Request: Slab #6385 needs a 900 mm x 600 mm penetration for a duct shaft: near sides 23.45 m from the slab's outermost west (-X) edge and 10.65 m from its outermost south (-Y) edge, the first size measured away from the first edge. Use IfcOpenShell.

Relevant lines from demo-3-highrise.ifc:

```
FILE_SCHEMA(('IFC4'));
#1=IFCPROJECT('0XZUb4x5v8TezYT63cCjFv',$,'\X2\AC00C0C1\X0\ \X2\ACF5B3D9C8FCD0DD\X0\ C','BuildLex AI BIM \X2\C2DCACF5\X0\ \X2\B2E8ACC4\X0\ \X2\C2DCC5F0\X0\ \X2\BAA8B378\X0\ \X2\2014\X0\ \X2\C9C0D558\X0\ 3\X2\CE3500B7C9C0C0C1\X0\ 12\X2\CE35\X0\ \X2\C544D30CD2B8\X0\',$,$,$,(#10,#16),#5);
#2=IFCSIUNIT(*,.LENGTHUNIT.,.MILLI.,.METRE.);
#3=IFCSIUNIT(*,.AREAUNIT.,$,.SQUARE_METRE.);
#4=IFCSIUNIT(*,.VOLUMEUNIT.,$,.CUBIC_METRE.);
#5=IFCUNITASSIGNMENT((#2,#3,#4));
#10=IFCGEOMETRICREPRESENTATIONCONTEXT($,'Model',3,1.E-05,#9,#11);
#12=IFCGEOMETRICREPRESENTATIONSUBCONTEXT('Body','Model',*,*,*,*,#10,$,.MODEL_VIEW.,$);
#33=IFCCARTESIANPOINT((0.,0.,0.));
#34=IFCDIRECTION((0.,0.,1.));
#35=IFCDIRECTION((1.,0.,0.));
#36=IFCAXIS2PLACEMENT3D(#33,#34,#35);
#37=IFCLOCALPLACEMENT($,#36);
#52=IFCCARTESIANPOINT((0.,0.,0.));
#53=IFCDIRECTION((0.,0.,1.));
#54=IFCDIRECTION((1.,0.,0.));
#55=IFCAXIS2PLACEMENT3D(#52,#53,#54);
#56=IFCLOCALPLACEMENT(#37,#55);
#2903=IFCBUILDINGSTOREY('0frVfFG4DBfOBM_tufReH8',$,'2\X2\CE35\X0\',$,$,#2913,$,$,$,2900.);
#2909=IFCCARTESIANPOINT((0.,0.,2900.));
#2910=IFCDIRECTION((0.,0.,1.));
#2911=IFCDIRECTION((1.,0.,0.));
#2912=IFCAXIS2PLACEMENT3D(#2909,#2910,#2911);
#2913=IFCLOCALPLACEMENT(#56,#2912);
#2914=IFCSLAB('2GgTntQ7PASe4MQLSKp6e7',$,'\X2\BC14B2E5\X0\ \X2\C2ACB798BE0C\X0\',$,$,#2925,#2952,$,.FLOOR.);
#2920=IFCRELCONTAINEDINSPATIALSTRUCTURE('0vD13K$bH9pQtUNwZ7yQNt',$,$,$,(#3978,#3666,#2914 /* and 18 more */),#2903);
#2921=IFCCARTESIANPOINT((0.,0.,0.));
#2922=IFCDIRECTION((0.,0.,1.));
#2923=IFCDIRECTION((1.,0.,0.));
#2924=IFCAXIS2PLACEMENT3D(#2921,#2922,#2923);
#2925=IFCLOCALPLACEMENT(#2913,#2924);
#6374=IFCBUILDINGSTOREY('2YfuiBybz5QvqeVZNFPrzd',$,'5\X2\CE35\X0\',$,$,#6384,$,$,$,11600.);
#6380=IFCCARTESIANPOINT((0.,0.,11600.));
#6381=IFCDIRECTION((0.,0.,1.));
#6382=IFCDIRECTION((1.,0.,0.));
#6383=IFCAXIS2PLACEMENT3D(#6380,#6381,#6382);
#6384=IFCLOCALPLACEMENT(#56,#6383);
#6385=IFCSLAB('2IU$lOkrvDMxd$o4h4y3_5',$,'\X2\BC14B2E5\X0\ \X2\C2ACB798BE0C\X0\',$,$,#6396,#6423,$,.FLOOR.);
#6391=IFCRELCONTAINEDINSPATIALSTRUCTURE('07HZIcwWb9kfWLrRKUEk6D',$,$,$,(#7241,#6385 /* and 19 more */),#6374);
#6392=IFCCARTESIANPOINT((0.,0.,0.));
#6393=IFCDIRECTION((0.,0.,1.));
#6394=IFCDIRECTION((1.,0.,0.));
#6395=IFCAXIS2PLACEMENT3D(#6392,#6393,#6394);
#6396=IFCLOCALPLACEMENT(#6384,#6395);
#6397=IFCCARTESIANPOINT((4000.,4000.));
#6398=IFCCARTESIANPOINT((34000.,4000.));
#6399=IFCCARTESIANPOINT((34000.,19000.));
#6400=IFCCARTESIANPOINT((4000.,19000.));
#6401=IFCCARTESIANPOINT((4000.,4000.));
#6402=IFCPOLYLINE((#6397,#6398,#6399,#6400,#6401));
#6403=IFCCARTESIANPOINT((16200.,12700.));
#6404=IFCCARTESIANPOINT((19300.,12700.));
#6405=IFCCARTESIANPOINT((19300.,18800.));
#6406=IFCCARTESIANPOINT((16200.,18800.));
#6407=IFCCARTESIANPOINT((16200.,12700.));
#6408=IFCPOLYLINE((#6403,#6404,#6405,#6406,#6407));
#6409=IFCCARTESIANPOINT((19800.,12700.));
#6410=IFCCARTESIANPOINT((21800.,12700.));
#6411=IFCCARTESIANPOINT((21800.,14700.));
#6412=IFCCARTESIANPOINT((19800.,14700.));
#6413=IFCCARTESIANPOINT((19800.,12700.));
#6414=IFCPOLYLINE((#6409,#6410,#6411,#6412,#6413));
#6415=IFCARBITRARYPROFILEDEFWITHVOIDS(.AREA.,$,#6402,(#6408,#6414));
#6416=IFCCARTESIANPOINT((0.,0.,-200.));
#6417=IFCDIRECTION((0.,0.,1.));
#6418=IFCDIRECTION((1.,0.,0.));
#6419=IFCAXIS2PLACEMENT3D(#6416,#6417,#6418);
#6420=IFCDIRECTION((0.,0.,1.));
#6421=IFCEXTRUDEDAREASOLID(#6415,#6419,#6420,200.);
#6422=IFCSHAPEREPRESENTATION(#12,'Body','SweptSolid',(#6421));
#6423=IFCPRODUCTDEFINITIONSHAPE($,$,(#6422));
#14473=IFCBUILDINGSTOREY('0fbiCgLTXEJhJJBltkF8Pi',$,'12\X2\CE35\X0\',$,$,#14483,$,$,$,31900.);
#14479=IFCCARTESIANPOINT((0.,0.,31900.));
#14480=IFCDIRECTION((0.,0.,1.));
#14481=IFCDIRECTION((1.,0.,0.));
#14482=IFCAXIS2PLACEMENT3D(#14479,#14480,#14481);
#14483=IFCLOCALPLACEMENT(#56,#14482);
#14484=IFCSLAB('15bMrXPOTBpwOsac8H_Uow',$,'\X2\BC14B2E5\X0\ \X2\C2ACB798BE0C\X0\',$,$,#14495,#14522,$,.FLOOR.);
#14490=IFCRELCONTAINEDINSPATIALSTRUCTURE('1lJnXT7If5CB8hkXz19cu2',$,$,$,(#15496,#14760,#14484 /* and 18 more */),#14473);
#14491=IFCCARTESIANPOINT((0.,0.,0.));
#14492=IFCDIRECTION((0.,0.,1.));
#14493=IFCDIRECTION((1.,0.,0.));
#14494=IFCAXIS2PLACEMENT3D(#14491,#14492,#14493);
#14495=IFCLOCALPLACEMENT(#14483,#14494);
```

```python
import numpy as np
import ifcopenshell
import ifcopenshell.api.feature
import ifcopenshell.api.geometry
import ifcopenshell.api.root
import ifcopenshell.geom
import ifcopenshell.util.placement
import ifcopenshell.util.representation
import ifcopenshell.util.shape
import ifcopenshell.util.unit

model = ifcopenshell.open("demo-3-highrise.ifc")
unit_scale = ifcopenshell.util.unit.calculate_unit_scale(model)
settings = ifcopenshell.geom.settings()


def volume(element):
    """Net volume in cubic metres, openings subtracted."""
    shape = ifcopenshell.geom.create_shape(settings, element)
    return ifcopenshell.util.shape.get_volume(shape.geometry)


slab = model.by_guid("2IU$lOkrvDMxd$o4h4y3_5")
before = volume(slab)

# Extent in the slab's own axes, in metres. The edges named are its -X and -Y sides.
slab_shape = ifcopenshell.geom.create_shape(settings, slab)
vertices = ifcopenshell.util.shape.get_vertices(slab_shape.geometry)
x_min, y_min, bottom = vertices.min(axis=0)
top = vertices[:, 2].max()

opening = ifcopenshell.api.root.create_entity(model, ifc_class="IfcOpeningElement", name="Duct shaft opening", predefined_type="OPENING")
context = ifcopenshell.util.representation.get_context(model, "Model", "Body", "MODEL_VIEW")
width, depth = 0.9, 0.6
outline = [(0.0, 0.0), (width, 0.0), (width, depth), (0.0, depth), (0.0, 0.0)]
# Overshoot both faces by 50 mm so the cut is clean.
shape = ifcopenshell.api.geometry.add_slab_representation(
    model, context=context, depth=top - bottom + 0.1, polyline=outline
)
ifcopenshell.api.geometry.assign_representation(model, product=opening, representation=shape)

matrix = ifcopenshell.util.placement.get_local_placement(slab.ObjectPlacement)
matrix[:, 3] = matrix @ np.append(np.array([x_min + 23.45, y_min + 10.65, bottom - 0.05]) / unit_scale, 1.0)
ifcopenshell.api.geometry.edit_object_placement(model, product=opening, matrix=matrix, is_si=False)
ifcopenshell.api.feature.add_feature(model, feature=opening, element=slab)

after = volume(slab)

print(f"slab volume {before:.3f} -> {after:.3f} m3")

model.write("demo-3-highrise_rev.ifc")
```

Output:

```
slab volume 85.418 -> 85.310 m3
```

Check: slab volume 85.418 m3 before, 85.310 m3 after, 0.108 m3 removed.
